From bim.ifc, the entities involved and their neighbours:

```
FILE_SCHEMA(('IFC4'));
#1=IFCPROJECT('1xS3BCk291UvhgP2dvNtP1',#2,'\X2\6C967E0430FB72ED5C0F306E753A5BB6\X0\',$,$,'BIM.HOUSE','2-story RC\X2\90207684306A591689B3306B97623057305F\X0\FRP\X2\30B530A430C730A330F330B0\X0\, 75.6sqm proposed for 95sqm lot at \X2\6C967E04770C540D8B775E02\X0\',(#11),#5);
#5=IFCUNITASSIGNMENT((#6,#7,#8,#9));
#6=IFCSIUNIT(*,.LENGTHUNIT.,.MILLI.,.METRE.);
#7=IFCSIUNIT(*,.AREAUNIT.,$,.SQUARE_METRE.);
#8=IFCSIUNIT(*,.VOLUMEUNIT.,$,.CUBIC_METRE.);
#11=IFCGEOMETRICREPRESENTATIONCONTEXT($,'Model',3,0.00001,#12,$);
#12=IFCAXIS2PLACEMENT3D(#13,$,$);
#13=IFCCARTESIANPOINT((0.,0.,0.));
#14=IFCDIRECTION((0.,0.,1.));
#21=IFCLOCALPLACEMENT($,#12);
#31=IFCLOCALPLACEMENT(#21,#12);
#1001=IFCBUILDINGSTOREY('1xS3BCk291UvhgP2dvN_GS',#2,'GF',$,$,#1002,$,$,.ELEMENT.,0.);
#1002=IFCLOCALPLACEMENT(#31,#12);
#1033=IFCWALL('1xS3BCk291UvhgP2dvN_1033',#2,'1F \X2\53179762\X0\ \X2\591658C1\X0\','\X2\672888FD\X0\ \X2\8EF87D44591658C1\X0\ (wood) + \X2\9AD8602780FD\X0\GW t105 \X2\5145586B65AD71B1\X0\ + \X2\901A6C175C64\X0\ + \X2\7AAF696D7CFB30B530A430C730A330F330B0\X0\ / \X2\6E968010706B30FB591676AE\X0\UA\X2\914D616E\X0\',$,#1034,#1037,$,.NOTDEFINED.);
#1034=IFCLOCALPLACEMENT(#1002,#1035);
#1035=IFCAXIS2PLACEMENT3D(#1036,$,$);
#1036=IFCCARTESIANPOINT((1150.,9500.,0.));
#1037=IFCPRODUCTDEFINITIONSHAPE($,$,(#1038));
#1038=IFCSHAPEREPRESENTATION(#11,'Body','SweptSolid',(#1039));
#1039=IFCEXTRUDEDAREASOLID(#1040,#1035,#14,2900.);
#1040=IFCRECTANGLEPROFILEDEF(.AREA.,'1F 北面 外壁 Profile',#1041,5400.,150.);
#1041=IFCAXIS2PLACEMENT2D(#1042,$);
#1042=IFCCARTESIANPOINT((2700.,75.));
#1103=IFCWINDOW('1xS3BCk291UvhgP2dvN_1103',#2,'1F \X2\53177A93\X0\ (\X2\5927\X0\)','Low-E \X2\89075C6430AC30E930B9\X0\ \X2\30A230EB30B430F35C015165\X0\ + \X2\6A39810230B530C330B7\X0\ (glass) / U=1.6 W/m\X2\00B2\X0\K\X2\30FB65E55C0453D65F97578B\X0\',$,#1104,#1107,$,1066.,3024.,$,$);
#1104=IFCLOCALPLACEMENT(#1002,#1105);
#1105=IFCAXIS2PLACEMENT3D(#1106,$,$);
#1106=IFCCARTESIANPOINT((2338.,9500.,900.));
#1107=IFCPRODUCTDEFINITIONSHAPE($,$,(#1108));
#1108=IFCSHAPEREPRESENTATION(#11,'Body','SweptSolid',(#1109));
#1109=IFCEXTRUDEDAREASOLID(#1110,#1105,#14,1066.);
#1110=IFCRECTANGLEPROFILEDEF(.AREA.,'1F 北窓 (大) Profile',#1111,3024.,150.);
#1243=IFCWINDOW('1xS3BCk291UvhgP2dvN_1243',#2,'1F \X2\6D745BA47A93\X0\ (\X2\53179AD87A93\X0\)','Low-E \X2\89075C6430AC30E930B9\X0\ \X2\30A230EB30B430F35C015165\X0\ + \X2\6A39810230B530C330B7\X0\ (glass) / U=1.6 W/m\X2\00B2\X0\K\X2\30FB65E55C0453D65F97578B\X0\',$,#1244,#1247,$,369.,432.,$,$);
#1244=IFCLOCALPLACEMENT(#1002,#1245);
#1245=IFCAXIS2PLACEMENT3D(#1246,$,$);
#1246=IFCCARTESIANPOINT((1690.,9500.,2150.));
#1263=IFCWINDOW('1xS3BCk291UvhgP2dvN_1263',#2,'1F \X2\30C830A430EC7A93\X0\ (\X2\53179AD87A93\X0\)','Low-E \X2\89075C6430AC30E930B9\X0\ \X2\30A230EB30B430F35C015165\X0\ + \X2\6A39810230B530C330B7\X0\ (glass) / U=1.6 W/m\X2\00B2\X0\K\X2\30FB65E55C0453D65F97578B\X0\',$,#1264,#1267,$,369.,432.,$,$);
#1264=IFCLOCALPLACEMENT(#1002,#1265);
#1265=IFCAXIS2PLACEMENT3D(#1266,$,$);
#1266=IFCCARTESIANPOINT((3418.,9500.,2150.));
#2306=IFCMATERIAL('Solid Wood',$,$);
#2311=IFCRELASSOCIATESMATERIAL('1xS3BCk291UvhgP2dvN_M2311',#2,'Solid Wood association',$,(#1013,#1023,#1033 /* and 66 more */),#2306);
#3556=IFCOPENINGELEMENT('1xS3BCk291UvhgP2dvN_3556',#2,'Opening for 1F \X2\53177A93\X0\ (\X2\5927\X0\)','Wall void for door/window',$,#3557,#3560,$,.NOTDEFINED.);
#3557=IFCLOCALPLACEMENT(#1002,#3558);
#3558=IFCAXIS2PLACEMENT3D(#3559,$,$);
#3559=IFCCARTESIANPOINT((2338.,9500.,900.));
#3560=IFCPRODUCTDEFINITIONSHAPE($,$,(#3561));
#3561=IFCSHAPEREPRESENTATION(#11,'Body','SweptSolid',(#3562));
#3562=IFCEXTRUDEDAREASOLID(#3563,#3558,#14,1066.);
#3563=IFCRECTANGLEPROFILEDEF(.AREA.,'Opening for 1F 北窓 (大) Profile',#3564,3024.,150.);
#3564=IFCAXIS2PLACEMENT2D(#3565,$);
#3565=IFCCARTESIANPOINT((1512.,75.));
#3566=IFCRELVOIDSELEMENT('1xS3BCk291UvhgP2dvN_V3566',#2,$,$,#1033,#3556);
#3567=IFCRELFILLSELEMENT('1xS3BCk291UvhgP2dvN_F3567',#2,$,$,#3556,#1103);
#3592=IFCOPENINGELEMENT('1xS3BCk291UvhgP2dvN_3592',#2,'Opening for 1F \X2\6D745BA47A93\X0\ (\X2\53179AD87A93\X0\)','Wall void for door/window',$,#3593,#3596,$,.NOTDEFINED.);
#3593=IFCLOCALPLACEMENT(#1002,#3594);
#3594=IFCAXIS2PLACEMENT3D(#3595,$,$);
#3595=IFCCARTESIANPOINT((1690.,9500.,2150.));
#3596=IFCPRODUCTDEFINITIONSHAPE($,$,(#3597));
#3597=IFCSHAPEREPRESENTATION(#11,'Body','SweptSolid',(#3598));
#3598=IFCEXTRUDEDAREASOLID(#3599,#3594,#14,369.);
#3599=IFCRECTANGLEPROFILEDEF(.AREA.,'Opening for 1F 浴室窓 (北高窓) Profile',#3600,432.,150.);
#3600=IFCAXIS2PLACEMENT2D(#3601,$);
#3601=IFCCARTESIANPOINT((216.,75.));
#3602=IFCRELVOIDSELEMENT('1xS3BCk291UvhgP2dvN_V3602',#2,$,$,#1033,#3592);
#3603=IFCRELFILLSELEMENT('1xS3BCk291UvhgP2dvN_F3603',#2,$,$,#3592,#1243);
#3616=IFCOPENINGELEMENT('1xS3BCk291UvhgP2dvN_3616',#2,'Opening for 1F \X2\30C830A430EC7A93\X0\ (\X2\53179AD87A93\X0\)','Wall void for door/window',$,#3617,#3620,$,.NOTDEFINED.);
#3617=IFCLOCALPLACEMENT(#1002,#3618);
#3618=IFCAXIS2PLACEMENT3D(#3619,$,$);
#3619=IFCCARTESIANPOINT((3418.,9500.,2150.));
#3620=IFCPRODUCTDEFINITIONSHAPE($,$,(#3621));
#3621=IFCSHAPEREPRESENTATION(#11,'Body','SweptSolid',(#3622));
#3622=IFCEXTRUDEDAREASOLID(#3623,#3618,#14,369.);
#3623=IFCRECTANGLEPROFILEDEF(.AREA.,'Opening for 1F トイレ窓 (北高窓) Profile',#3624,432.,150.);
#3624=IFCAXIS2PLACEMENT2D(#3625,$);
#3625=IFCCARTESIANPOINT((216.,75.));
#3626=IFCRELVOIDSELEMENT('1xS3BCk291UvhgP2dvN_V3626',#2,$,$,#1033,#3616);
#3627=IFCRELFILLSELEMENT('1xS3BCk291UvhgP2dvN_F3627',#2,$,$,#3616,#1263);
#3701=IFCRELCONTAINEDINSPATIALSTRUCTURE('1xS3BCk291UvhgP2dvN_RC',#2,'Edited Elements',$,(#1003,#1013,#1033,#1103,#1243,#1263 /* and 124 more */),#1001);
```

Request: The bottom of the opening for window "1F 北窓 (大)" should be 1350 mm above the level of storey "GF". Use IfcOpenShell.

```python
import numpy as np
import ifcopenshell
import ifcopenshell.api.geometry
import ifcopenshell.geom
import ifcopenshell.util.element
import ifcopenshell.util.placement
import ifcopenshell.util.shape
import ifcopenshell.util.unit

model = ifcopenshell.open("bim.ifc")
unit_scale = ifcopenshell.util.unit.calculate_unit_scale(model)

window = model.by_id(1103)
opening = window.FillsVoids[0].RelatingOpeningElement
storey = ifcopenshell.util.element.get_container(window, ifc_class="IfcBuildingStorey")
level = ifcopenshell.util.placement.get_local_placement(storey.ObjectPlacement)[2, 3]

# The opening's origin need not be at the sill, so measure its lowest point.
shape = ifcopenshell.geom.create_shape(ifcopenshell.geom.settings(), opening)
bottom = ifcopenshell.util.shape.get_shape_bottom_elevation(shape, shape.geometry) / unit_scale
dz = level + 1350.0 - bottom

shift = np.array([0.0, 0.0, dz])
# The window is not placed relative to its opening, so move both.
for product in (opening, window):
    matrix = ifcopenshell.util.placement.get_local_placement(product.ObjectPlacement)
    matrix[:3, 3] += shift
    ifcopenshell.api.geometry.edit_object_placement(model, product=product, matrix=matrix, is_si=False)

print(f"moved by {dz * unit_scale:+.3f} m")

model.write("bim_rev.ifc")
```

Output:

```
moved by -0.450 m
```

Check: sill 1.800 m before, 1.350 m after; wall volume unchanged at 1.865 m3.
